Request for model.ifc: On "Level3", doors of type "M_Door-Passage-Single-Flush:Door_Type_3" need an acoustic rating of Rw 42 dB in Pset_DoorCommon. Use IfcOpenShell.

First a look at what the model holds.

```python
import ifcopenshell
import ifcopenshell.util.element

model = ifcopenshell.open("model.ifc")
print(model.schema)
storey = next(s for s in model.by_type("IfcBuildingStorey") if s.Name == "Level3")
doors = [e for e in ifcopenshell.util.element.get_decomposition(storey) if e.is_a("IfcDoor")]
seen = {}
for e in doors:
    element_type = ifcopenshell.util.element.get_type(e)
    key = (element_type.Name if element_type != e and element_type else None, ifcopenshell.util.element.get_pset(e, "Pset_DoorCommon", "AcousticRating"))
    seen[key] = seen.get(key, 0) + 1
for (name, value), count in sorted(seen.items(), key=str):
    print(count, "x", name, "|", value)
```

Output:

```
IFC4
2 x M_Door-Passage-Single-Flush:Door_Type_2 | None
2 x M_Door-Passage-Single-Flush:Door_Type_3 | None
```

```python
import ifcopenshell
import ifcopenshell.api.pset
import ifcopenshell.util.element

model = ifcopenshell.open("model.ifc")

storey = next(s for s in model.by_type("IfcBuildingStorey") if s.Name == "Level3")
doors = [e for e in ifcopenshell.util.element.get_decomposition(storey) if e.is_a("IfcDoor")]

count = 0
for e in doors:
    element_type = ifcopenshell.util.element.get_type(e)
    if element_type in (None, e) or element_type.Name != "M_Door-Passage-Single-Flush:Door_Type_3":
        continue
    # add_pset returns the element's existing set when there is one.
    pset = ifcopenshell.api.pset.add_pset(model, product=e, name="Pset_DoorCommon")
    ifcopenshell.api.pset.edit_pset(model, pset=pset, properties={"AcousticRating": "Rw 42 dB"})
    count += 1

print(count, "doors updated")

model.write("model_updated.ifc")
```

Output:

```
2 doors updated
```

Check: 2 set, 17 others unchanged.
